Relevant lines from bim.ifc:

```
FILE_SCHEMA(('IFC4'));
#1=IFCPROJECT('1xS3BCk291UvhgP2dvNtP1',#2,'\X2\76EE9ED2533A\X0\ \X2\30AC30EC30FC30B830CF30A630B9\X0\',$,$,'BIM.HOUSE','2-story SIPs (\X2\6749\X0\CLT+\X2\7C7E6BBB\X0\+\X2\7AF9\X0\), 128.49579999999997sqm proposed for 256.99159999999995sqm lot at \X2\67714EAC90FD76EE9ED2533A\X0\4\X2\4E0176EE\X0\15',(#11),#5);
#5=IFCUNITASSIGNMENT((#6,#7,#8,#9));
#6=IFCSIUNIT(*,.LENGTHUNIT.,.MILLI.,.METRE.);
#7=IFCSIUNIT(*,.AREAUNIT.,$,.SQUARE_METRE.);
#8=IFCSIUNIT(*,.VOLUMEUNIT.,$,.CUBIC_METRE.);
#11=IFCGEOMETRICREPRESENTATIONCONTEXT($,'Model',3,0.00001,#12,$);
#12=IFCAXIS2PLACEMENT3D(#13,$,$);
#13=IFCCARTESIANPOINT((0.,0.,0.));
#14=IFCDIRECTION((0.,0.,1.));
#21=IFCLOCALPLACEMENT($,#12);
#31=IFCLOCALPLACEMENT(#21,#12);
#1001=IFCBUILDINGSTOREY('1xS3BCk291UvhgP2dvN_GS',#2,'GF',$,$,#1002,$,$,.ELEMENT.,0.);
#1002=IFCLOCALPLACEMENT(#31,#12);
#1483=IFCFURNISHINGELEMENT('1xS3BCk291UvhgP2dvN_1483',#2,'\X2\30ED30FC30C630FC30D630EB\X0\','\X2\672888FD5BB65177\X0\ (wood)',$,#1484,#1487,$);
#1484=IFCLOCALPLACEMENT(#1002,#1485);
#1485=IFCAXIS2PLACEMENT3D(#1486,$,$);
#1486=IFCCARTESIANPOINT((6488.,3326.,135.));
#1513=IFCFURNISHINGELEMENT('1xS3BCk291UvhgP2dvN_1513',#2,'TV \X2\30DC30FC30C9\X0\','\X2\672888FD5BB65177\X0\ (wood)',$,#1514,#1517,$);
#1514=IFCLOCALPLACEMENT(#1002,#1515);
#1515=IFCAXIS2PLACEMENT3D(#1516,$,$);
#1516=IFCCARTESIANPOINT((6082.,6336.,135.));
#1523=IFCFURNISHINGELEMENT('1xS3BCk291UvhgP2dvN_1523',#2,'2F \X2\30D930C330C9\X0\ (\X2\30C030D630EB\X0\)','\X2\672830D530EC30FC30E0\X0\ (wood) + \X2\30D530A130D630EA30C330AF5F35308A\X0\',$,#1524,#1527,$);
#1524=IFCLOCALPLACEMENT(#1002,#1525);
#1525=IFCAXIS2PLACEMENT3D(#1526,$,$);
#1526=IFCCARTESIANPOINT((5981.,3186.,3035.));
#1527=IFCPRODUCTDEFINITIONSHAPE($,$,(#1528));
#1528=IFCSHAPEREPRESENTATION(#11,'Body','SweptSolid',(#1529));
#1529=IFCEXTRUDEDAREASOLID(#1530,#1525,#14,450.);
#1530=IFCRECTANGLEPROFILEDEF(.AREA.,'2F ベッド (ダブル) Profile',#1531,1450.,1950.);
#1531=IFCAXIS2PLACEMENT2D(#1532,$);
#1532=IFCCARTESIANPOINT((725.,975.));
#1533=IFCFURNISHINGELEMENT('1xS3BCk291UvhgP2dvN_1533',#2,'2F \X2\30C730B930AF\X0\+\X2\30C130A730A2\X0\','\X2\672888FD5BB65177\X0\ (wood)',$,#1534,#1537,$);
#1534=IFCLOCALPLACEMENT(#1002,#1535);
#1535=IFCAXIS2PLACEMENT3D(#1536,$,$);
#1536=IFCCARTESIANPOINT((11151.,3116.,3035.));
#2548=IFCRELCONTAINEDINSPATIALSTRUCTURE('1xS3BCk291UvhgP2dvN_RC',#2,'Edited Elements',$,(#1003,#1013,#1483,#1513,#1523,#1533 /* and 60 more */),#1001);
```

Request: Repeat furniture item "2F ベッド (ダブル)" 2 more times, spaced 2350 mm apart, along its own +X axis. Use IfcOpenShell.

```python
import ifcopenshell
import ifcopenshell.api.geometry
import ifcopenshell.api.root
import ifcopenshell.util.element
import ifcopenshell.util.placement
import ifcopenshell.util.unit

model = ifcopenshell.open("bim.ifc")
unit_scale = ifcopenshell.util.unit.calculate_unit_scale(model)


def reuse_history(source, copy):
    """copy_class also copies each property set's owner history, people and application; keep the originals."""
    for rel in copy.IsDefinedBy:
        if rel.is_a("IfcRelDefinesByProperties") and (history := rel.RelatingPropertyDefinition.OwnerHistory):
            rel.RelatingPropertyDefinition.OwnerHistory = source.OwnerHistory
            ifcopenshell.util.element.remove_deep2(model, history)


source = model.by_guid("1xS3BCk291UvhgP2dvN_1523")
base = ifcopenshell.util.placement.get_local_placement(source.ObjectPlacement)
step = base[:3, 0] * 2.35 / unit_scale

for i in range(1, 3):
    copy = ifcopenshell.api.root.copy_class(model, product=source)
    copy.Representation = ifcopenshell.util.element.copy_deep(
        model, source.Representation, exclude=["IfcGeometricRepresentationContext", "IfcRepresentationMap"]
    )
    reuse_history(source, copy)
    matrix = base.copy()
    matrix[:3, 3] += i * step
    print("added at", matrix[:3, 3].round(3) + 0.0)
    ifcopenshell.api.geometry.edit_object_placement(model, product=copy, matrix=matrix, is_si=False)

model.write("bim_edited.ifc")
```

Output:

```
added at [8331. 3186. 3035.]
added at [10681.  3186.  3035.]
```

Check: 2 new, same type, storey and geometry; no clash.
